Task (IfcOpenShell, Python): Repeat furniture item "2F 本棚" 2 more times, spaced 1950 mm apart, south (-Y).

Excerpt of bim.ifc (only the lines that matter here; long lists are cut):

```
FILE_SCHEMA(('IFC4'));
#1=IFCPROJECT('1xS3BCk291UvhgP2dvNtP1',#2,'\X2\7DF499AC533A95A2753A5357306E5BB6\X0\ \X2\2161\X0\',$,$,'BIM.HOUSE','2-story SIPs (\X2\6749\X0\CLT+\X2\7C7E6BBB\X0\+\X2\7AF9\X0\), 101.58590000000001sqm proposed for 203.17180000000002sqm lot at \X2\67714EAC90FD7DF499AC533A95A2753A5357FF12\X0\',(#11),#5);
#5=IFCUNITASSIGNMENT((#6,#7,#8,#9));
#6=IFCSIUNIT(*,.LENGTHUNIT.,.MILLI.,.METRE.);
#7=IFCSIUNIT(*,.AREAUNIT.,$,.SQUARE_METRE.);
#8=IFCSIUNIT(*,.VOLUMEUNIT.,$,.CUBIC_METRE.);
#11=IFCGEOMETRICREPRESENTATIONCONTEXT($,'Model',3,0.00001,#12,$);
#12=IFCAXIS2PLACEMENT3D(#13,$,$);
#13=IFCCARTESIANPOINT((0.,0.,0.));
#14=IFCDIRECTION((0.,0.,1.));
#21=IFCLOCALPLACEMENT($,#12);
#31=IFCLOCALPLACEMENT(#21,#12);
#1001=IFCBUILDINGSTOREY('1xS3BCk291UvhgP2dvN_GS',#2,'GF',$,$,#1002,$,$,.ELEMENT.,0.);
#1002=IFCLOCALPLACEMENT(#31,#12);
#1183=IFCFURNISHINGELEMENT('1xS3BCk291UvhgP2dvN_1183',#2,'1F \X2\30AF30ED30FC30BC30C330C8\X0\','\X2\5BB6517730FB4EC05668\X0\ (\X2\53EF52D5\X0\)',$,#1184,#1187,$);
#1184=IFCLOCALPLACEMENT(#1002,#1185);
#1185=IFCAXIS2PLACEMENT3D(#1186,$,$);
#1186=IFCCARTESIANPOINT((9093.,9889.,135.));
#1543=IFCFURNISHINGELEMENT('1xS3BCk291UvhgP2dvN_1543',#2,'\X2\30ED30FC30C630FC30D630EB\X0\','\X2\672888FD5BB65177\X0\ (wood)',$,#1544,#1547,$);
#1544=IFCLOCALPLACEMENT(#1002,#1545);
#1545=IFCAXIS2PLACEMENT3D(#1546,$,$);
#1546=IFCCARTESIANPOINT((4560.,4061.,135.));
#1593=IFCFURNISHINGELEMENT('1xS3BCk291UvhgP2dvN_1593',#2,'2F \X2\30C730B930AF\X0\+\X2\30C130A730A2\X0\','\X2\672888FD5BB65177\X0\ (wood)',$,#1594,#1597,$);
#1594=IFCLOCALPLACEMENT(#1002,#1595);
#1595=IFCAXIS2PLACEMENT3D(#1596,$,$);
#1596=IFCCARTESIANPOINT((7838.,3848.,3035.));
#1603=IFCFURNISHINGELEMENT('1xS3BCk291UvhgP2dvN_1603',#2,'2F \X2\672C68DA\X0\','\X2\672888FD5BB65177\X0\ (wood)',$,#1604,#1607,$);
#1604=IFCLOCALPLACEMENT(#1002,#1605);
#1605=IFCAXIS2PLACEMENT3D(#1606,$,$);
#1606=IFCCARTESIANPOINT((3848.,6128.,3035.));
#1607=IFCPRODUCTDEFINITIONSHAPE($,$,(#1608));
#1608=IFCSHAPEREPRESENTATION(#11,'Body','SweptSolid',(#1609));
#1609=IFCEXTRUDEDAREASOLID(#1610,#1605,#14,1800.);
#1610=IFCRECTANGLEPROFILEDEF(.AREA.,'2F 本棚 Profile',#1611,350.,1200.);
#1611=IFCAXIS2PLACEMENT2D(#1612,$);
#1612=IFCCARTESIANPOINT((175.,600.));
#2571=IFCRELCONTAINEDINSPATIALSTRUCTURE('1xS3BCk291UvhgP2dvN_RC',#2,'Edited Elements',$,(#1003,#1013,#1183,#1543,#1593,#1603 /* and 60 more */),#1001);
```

```python
import numpy as np
import ifcopenshell
import ifcopenshell.api.geometry
import ifcopenshell.api.root
import ifcopenshell.util.element
import ifcopenshell.util.placement

model = ifcopenshell.open("bim.ifc")


def reuse_history(source, copy):
    """copy_class also copies each property set's owner history, people and application; keep the originals."""
    for rel in copy.IsDefinedBy:
        if rel.is_a("IfcRelDefinesByProperties") and (history := rel.RelatingPropertyDefinition.OwnerHistory):
            rel.RelatingPropertyDefinition.OwnerHistory = source.OwnerHistory
            ifcopenshell.util.element.remove_deep2(model, history)


source = model.by_id(1603)
base = ifcopenshell.util.placement.get_local_placement(source.ObjectPlacement)
step = np.array([0.0, -1.0, 0.0]) * 1950.0

for i in range(1, 3):
    copy = ifcopenshell.api.root.copy_class(model, product=source)
    copy.Representation = ifcopenshell.util.element.copy_deep(
        model, source.Representation, exclude=["IfcGeometricRepresentationContext", "IfcRepresentationMap"]
    )
    reuse_history(source, copy)
    matrix = base.copy()
    matrix[:3, 3] += i * step
    print("added at", matrix[:3, 3].round(3) + 0.0)
    ifcopenshell.api.geometry.edit_object_placement(model, product=copy, matrix=matrix, is_si=False)

model.write("bim_edited.ifc")
```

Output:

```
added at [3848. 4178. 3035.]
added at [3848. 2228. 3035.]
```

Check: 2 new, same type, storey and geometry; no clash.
